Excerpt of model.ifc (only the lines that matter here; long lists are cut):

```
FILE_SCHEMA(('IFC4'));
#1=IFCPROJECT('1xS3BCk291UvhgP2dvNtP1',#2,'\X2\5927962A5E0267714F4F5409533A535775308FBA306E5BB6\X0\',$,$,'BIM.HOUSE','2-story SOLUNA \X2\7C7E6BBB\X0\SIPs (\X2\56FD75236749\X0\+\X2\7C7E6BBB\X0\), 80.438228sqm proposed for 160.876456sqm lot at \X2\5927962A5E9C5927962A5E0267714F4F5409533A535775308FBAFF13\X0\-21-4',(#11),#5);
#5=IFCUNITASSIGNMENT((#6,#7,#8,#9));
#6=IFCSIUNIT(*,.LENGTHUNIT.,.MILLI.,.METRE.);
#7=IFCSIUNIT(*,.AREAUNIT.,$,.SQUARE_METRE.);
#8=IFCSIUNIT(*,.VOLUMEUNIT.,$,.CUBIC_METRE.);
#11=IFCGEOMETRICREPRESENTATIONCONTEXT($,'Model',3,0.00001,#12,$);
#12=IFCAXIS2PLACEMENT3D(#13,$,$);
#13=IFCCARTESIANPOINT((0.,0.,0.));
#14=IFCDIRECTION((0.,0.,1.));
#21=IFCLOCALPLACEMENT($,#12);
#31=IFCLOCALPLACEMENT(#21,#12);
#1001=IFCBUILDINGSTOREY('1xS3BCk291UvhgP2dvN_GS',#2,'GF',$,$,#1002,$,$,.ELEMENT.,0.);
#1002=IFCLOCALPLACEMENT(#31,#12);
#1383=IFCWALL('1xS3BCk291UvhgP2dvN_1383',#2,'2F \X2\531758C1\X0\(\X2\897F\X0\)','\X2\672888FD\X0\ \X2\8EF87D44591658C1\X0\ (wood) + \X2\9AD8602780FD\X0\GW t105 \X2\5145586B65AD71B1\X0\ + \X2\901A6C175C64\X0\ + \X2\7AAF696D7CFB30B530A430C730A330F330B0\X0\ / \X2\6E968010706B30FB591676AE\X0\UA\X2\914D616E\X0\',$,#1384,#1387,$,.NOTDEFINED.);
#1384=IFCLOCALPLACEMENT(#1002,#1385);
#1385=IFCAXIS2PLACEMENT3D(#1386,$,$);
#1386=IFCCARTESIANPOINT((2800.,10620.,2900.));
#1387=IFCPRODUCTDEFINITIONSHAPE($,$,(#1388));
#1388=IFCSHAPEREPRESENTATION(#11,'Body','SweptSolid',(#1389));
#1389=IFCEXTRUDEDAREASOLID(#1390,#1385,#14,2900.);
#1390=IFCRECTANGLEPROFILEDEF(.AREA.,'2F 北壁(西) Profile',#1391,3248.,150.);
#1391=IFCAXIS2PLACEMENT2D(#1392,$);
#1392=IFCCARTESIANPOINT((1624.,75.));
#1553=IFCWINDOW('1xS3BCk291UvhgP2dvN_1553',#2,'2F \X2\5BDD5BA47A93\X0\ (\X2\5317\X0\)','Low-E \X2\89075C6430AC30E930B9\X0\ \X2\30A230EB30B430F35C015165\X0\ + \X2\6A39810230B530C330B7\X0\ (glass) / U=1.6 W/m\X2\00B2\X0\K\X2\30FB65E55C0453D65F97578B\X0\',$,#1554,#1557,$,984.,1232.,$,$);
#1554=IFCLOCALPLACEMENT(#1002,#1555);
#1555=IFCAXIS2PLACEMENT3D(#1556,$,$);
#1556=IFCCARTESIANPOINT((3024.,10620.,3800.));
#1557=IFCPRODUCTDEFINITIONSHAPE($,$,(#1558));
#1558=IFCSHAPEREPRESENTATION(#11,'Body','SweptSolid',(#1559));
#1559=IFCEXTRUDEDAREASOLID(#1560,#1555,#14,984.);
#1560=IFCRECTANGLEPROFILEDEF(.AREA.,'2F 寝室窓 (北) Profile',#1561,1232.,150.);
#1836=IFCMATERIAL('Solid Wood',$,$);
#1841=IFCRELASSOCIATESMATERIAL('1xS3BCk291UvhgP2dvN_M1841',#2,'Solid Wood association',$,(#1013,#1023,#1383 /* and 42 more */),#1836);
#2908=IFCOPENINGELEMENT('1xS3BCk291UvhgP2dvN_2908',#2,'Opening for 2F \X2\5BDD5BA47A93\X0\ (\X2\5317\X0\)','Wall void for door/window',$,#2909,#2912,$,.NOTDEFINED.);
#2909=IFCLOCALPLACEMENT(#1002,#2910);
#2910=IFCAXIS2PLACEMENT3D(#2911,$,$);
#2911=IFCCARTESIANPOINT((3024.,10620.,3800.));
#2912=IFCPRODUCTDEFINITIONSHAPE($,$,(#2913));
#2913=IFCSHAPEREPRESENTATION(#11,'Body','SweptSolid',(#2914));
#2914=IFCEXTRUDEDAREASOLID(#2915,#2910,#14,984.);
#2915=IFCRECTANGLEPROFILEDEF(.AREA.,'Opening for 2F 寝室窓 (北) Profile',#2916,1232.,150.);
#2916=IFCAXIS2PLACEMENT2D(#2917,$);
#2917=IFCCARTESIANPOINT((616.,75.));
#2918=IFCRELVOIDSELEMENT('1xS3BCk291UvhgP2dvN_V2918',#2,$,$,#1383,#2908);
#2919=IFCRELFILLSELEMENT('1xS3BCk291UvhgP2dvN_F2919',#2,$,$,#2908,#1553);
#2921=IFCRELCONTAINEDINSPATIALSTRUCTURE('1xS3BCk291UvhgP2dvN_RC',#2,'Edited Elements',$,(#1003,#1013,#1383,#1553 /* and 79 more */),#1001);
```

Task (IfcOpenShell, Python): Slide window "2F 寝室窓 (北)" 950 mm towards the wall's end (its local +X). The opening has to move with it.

```python
import ifcopenshell
import ifcopenshell.api.geometry
import ifcopenshell.util.placement

model = ifcopenshell.open("model.ifc")

window = model.by_guid("1xS3BCk291UvhgP2dvN_1553")
opening = window.FillsVoids[0].RelatingOpeningElement
wall = opening.VoidsElements[0].RelatingBuildingElement

wall_matrix = ifcopenshell.util.placement.get_local_placement(wall.ObjectPlacement)
shift = wall_matrix[:3, 0] * 950.0
before = ifcopenshell.util.placement.get_local_placement(window.ObjectPlacement)[:3, 3].copy()

# The window is not placed relative to its opening, so move both.
for product in (opening, window):
    matrix = ifcopenshell.util.placement.get_local_placement(product.ObjectPlacement)
    matrix[:3, 3] += shift
    ifcopenshell.api.geometry.edit_object_placement(model, product=product, matrix=matrix, is_si=False)

after = ifcopenshell.util.placement.get_local_placement(window.ObjectPlacement)[:3, 3]
print("window moved by", (after - before).round(3) + 0.0)

model.write("model_rev.ifc")
```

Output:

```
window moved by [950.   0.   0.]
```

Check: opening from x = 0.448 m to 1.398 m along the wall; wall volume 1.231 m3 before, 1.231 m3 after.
